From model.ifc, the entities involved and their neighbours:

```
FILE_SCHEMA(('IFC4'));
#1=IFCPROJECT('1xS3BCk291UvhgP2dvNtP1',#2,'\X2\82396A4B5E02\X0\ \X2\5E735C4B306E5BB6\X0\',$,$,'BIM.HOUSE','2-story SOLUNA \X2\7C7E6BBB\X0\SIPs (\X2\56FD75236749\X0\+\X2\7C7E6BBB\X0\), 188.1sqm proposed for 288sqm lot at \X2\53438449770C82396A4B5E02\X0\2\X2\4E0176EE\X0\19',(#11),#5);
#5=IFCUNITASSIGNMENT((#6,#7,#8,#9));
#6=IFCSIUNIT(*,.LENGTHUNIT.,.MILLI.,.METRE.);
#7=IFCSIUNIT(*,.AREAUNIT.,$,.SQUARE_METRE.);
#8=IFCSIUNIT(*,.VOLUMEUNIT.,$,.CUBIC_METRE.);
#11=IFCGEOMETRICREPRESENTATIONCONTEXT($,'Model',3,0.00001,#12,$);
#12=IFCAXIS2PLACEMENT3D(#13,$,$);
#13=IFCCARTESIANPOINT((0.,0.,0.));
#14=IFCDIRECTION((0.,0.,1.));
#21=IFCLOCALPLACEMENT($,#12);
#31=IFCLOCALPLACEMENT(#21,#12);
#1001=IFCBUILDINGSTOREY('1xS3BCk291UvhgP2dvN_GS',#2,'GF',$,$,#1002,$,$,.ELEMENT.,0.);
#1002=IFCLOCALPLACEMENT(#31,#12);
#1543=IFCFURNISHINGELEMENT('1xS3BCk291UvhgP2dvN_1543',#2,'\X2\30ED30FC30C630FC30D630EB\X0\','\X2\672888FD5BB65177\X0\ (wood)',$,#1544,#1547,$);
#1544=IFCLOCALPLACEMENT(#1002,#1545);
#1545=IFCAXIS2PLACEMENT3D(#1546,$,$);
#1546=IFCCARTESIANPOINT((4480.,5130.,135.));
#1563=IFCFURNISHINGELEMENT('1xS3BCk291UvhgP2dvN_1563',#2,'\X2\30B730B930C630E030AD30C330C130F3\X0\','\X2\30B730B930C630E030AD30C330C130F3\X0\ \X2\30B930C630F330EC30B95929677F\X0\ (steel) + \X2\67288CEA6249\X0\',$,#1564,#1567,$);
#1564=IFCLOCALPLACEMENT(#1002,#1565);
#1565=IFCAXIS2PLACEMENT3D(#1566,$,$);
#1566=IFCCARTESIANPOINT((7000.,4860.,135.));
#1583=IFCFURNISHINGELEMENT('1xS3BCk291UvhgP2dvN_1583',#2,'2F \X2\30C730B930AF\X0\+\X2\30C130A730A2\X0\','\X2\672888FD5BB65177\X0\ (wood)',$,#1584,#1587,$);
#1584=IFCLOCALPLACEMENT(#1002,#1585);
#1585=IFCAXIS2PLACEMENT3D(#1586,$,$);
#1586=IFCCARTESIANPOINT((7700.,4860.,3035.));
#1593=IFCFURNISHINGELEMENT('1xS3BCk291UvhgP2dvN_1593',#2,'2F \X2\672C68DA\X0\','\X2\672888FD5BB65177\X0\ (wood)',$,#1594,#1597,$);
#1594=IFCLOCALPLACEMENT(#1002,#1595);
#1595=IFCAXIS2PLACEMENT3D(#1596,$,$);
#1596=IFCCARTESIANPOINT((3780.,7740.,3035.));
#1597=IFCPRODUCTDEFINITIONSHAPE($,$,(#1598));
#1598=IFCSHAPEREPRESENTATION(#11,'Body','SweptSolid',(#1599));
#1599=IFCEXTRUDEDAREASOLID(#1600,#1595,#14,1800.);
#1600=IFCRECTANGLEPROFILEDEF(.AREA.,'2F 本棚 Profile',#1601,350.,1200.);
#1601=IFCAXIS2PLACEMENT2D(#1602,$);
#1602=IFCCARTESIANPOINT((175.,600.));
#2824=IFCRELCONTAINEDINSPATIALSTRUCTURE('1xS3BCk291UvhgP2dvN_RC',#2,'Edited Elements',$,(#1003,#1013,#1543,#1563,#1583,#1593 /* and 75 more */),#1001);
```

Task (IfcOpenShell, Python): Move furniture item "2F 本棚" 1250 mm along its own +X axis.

```python
import ifcopenshell
import ifcopenshell.api.geometry
import ifcopenshell.util.placement
import ifcopenshell.util.unit

model = ifcopenshell.open("model.ifc")
unit_scale = ifcopenshell.util.unit.calculate_unit_scale(model)

item = model.by_guid("1xS3BCk291UvhgP2dvN_1593")
matrix = ifcopenshell.util.placement.get_local_placement(item.ObjectPlacement)
matrix[:3, 3] += matrix[:3, 0] * 1.25 / unit_scale
ifcopenshell.api.geometry.edit_object_placement(model, product=item, matrix=matrix, is_si=False)

print(ifcopenshell.util.placement.get_local_placement(item.ObjectPlacement).round(3) + 0.0)

model.write("model_v2.ifc")
```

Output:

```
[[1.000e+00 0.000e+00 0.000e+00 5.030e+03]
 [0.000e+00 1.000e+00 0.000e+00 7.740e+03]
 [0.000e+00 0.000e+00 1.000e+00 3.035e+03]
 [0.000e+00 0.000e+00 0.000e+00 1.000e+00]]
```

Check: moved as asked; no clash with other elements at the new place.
